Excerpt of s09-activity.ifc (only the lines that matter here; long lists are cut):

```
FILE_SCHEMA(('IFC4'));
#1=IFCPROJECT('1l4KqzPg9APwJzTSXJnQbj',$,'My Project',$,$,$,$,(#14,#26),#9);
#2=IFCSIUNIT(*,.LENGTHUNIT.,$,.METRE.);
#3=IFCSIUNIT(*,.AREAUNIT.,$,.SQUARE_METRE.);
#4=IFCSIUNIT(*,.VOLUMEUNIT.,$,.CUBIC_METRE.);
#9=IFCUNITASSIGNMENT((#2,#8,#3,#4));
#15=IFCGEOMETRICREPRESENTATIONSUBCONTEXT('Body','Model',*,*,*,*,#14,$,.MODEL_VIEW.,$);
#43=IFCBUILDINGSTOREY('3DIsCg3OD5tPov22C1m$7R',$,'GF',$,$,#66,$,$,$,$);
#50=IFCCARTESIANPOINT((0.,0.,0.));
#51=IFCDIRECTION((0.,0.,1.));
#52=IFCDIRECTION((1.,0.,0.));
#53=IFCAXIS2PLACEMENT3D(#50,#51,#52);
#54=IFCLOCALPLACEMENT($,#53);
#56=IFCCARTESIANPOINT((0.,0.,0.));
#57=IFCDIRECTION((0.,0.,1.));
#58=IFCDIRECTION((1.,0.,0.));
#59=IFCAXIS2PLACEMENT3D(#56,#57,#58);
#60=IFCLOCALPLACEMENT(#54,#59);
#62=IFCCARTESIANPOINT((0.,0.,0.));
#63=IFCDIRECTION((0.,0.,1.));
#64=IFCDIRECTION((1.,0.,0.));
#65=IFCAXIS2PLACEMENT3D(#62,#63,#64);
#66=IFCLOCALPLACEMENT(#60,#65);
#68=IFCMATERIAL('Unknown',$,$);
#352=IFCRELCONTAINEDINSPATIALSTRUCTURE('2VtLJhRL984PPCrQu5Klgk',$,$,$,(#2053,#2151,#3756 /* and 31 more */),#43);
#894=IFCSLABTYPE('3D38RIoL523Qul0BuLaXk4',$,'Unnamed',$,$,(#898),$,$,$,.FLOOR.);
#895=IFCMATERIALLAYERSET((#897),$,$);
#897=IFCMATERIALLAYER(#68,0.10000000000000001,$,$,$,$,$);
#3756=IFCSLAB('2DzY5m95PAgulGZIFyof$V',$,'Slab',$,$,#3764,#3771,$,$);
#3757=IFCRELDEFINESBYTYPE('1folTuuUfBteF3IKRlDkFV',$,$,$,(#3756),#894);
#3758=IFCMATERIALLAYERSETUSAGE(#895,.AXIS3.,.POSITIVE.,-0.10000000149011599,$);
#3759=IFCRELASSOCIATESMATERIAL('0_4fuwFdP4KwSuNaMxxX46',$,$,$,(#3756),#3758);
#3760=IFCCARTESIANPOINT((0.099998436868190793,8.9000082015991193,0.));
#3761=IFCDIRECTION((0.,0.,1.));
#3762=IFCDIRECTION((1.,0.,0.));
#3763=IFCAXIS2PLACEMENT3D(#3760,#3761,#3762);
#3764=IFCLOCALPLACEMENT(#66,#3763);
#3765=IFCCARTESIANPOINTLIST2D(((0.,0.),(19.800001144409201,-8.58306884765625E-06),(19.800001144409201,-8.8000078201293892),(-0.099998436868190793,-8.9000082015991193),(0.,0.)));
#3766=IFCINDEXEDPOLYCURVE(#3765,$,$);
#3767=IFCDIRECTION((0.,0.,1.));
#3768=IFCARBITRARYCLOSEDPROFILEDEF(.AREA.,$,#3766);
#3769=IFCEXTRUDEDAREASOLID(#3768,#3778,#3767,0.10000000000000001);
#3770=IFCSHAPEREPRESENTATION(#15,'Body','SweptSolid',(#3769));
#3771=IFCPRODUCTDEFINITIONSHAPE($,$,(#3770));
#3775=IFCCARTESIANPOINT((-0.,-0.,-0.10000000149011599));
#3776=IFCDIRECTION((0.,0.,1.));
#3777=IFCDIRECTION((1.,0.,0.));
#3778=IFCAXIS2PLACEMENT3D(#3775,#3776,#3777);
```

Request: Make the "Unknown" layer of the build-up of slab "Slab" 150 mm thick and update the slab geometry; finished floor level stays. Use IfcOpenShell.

```python
import ifcopenshell
import ifcopenshell.util.element
import ifcopenshell.util.representation
import ifcopenshell.util.unit

model = ifcopenshell.open("s09-activity.ifc")
unit_scale = ifcopenshell.util.unit.calculate_unit_scale(model)

layer_set = model.by_id(895)
layer = next(l for l in layer_set.MaterialLayers if l.Material and l.Material.Name == "Unknown")
change = 0.15 / unit_scale - layer.LayerThickness
layer.LayerThickness += change

# Geometry does not follow the layer set by itself.
slabs = [e for e in ifcopenshell.util.element.get_elements_by_material(model, layer_set) if e.is_a("IfcSlab")]
for slab in sorted(slabs, key=lambda e: e.id()):
    body = ifcopenshell.util.representation.get_representation(slab, "Model", "Body")
    solid = body.Items[0]
    old_depth = solid.Depth
    solid.Depth += change
    # Extruded upwards: lower the start of the extrusion so the top stays.
    x, y, z = solid.Position.Location.Coordinates
    solid.Position.Location = model.createIfcCartesianPoint((x, y, z - change))
    print(slab.id(), f"{old_depth:g} -> {solid.Depth:g}")

# The layers are counted up from the underside, which has moved.
for usage in {ifcopenshell.util.element.get_material(slab) for slab in slabs}:
    usage.OffsetFromReferenceLine -= change

model.write("s09-activity_updated.ifc")
```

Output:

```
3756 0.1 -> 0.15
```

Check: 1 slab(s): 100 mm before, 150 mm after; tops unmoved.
